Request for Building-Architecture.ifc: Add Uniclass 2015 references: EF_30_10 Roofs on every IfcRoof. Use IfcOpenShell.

First a look at what the model holds.

```python
import ifcopenshell

model = ifcopenshell.open("Building-Architecture.ifc")
print(model.schema)
print("classifications:", [c.Name for c in model.by_type("IfcClassification")])
for ifc_class in ("IfcDoor", "IfcRoof", "IfcStair", "IfcWall", "IfcWindow"):
    print(ifc_class, len(model.by_type(ifc_class)))
```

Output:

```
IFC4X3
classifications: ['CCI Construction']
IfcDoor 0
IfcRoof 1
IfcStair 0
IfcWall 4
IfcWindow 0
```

```python
import ifcopenshell
import ifcopenshell.api.classification

model = ifcopenshell.open("Building-Architecture.ifc")

system = ifcopenshell.api.classification.add_classification(model, classification="Uniclass 2015")

codes = {
    "IfcRoof": ("EF_30_10", "Roofs"),
}
for ifc_class, (code, name) in codes.items():
    products = model.by_type(ifc_class)
    ifcopenshell.api.classification.add_reference(
        model, products=products, classification=system, identification=code, name=name
    )
    print(code, len(products))

model.write("Building-Architecture_v2.ifc")
```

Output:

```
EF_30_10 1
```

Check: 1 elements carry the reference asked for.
